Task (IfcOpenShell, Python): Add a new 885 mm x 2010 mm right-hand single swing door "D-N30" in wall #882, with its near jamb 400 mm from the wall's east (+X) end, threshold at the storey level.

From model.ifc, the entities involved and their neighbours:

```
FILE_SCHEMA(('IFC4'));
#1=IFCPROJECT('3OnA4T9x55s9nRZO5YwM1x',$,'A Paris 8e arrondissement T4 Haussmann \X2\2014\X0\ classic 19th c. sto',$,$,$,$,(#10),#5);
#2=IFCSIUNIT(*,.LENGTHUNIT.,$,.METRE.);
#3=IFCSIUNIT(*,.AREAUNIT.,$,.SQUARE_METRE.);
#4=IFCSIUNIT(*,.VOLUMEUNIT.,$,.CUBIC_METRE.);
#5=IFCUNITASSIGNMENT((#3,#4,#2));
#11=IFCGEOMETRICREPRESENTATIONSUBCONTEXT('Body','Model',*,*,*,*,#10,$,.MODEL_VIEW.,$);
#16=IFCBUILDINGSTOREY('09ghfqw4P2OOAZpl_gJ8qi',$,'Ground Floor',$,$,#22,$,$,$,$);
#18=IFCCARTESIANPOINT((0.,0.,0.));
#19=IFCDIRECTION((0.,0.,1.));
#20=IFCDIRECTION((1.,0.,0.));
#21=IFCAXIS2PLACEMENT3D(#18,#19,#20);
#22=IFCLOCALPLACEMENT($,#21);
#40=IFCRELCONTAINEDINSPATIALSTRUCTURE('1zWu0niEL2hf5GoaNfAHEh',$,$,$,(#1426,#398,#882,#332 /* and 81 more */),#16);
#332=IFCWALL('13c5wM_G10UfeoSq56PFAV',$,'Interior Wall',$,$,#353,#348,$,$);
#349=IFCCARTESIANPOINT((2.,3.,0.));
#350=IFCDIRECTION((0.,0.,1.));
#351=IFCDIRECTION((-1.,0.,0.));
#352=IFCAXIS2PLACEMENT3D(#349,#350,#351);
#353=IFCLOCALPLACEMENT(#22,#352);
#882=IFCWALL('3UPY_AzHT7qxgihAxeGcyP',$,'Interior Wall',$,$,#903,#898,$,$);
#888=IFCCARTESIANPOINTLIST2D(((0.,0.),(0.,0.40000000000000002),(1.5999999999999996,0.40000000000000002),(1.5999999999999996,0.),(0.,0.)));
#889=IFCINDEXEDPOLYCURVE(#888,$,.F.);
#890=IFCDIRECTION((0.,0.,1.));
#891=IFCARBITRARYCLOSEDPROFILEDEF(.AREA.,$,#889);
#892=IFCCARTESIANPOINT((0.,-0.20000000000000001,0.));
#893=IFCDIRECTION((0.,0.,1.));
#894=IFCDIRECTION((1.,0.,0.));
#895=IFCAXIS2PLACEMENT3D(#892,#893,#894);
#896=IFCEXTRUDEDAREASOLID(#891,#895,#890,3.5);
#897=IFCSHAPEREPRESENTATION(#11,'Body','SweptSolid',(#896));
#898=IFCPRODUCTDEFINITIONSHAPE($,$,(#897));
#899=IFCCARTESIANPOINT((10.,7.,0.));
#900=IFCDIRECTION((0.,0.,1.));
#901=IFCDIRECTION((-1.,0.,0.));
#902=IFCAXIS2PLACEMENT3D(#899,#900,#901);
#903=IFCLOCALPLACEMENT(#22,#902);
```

```python
import numpy as np
import ifcopenshell
import ifcopenshell.api.feature
import ifcopenshell.api.geometry
import ifcopenshell.api.root
import ifcopenshell.api.spatial
import ifcopenshell.geom
import ifcopenshell.util.element
import ifcopenshell.util.placement
import ifcopenshell.util.representation
import ifcopenshell.util.shape
import ifcopenshell.util.unit

model = ifcopenshell.open("model.ifc")
unit_scale = ifcopenshell.util.unit.calculate_unit_scale(model)
settings = ifcopenshell.geom.settings()


def volume(element):
    """Net volume in cubic metres, openings subtracted."""
    shape = ifcopenshell.geom.create_shape(settings, element)
    return ifcopenshell.util.shape.get_volume(shape.geometry)


wall = model.by_guid("3UPY_AzHT7qxgihAxeGcyP")
storey = ifcopenshell.util.element.get_container(wall, ifc_class="IfcBuildingStorey")
context = ifcopenshell.util.representation.get_context(model, "Model", "Body", "MODEL_VIEW")
before = volume(wall)

width, height, from_end, sill = 0.885, 2.01, 0.4, 0.0  # metres

# The wall runs along its own X axis, and the end named is its -X end.
wall_shape = ifcopenshell.geom.create_shape(settings, wall)
x, y, z = ifcopenshell.util.shape.get_vertices(wall_shape.geometry).T
start = x.min() + from_end
face, thickness = float(y.min()), float(y.max() - y.min())
wall_matrix = ifcopenshell.util.placement.get_local_placement(wall.ObjectPlacement)
level = ifcopenshell.util.placement.get_local_placement(storey.ObjectPlacement)[2, 3]


def in_wall(x, y):
    """Placement at x, y metres in the wall's axes, at sill height."""
    matrix = wall_matrix.copy()
    matrix[:, 3] = wall_matrix @ np.array([x / unit_scale, y / unit_scale, 0.0, 1.0])
    matrix[2, 3] = level + sill / unit_scale
    return matrix


# Opening: a box that overshoots both wall faces by 50 mm.
opening = ifcopenshell.api.root.create_entity(model, ifc_class="IfcOpeningElement", predefined_type="OPENING")
box = ifcopenshell.api.geometry.add_wall_representation(
    model, context=context, length=width, height=height, thickness=thickness + 0.1
)
ifcopenshell.api.geometry.assign_representation(model, product=opening, representation=box)
ifcopenshell.api.geometry.edit_object_placement(model, product=opening, matrix=in_wall(start, face - 0.05), is_si=False)
ifcopenshell.api.feature.add_feature(model, feature=opening, element=wall)

door = ifcopenshell.api.root.create_entity(model, ifc_class="IfcDoor", name="D-N30", predefined_type="DOOR")
door.OverallWidth, door.OverallHeight = width / unit_scale, height / unit_scale
door.OperationType = "SINGLE_SWING_RIGHT"
body = ifcopenshell.api.geometry.add_door_representation(
    model,
    context=context,
    overall_width=door.OverallWidth,
    overall_height=door.OverallHeight,
    operation_type="SINGLE_SWING_RIGHT",
    lining_properties={"LiningDepth": thickness / unit_scale, "ThresholdDepth": thickness / unit_scale},
)
ifcopenshell.api.geometry.assign_representation(model, product=door, representation=body)
ifcopenshell.api.spatial.assign_container(model, products=[door], relating_structure=storey)
ifcopenshell.api.feature.add_filling(model, opening=opening, element=door)

# The lining spans the wall, so the door starts at the wall face.
ifcopenshell.api.geometry.edit_object_placement(model, product=door, matrix=in_wall(start, face), is_si=False)

after = volume(wall)

print(f"wall volume {before:.3f} -> {after:.3f} m3")

model.write("model_edited.ifc")
```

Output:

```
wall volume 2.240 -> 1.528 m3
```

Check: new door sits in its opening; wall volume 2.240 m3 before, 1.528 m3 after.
